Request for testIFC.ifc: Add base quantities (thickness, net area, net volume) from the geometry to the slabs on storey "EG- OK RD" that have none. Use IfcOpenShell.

First a look at what the model holds.

```python
import ifcopenshell
import ifcopenshell.util.element
import ifcopenshell.util.unit

model = ifcopenshell.open("testIFC.ifc")
print(model.schema)
for unit_type in ("LENGTHUNIT", "AREAUNIT", "VOLUMEUNIT"):
    print(unit_type, ifcopenshell.util.unit.calculate_unit_scale(model, unit_type))
storey = next(s for s in model.by_type("IfcBuildingStorey") if s.Name == "EG- OK RD")
slabs = [e for e in ifcopenshell.util.element.get_decomposition(storey) if e.is_a("IfcSlab")]
for e in sorted(slabs, key=lambda e: e.id()):
    print(e.id(), e.is_a(), e.Name, list(ifcopenshell.util.element.get_psets(e, qtos_only=True)), sep=" | ")
```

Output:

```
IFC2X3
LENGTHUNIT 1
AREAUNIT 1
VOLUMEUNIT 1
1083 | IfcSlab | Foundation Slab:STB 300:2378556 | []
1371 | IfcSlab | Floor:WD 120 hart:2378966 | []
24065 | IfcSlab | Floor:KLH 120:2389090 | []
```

```python
import ifcopenshell
import ifcopenshell.api.pset
import ifcopenshell.geom
import ifcopenshell.util.element
import ifcopenshell.util.shape
import ifcopenshell.util.unit

model = ifcopenshell.open("testIFC.ifc")
unit_scale = ifcopenshell.util.unit.calculate_unit_scale(model)
area_scale = ifcopenshell.util.unit.calculate_unit_scale(model, "AREAUNIT")
volume_scale = ifcopenshell.util.unit.calculate_unit_scale(model, "VOLUMEUNIT")
settings = ifcopenshell.geom.settings()

storey = next(s for s in model.by_type("IfcBuildingStorey") if s.Name == "EG- OK RD")
slabs = [e for e in ifcopenshell.util.element.get_decomposition(storey) if e.is_a("IfcSlab")]

for e in sorted(slabs, key=lambda e: e.id()):
    if ifcopenshell.util.element.get_psets(e, qtos_only=True, should_inherit=False):
        continue
    # Geometry comes back in metres, in the element's own axes.
    shape = ifcopenshell.geom.create_shape(settings, e)
    values = {
        "Width": ifcopenshell.util.shape.get_z(shape.geometry) / unit_scale,
        "NetArea": ifcopenshell.util.shape.get_footprint_area(shape.geometry) / area_scale,
        "NetVolume": ifcopenshell.util.shape.get_volume(shape.geometry) / volume_scale,
    }
    qto = ifcopenshell.api.pset.add_qto(model, product=e, name="BaseQuantities")
    ifcopenshell.api.pset.edit_qto(model, qto=qto, properties=values)
    print(e.id(), {k: round(v, 3) for k, v in values.items()})

model.write("testIFC_v2.ifc")
```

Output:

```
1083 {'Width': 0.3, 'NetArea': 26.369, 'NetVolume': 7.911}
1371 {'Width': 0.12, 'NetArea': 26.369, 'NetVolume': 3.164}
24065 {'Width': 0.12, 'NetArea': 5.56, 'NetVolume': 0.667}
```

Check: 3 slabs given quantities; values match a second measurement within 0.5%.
